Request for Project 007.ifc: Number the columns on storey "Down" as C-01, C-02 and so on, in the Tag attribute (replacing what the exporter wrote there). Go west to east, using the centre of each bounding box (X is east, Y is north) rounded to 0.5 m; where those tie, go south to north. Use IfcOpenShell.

First a look at what the model holds.

```python
import ifcopenshell
import ifcopenshell.util.element
import ifcopenshell.util.placement

model = ifcopenshell.open("Project 007.ifc")
print(model.schema)
storey = next(s for s in model.by_type("IfcBuildingStorey") if s.Name == "Down")
columns = [e for e in ifcopenshell.util.element.get_decomposition(storey) if e.is_a("IfcColumn")]
for e in sorted(columns, key=lambda e: e.id()):
    origin = ifcopenshell.util.placement.get_local_placement(e.ObjectPlacement)[:3, 3]
    print(e.id(), e.Tag, e.Name, origin.round(2) + 0.0, sep=" | ")
```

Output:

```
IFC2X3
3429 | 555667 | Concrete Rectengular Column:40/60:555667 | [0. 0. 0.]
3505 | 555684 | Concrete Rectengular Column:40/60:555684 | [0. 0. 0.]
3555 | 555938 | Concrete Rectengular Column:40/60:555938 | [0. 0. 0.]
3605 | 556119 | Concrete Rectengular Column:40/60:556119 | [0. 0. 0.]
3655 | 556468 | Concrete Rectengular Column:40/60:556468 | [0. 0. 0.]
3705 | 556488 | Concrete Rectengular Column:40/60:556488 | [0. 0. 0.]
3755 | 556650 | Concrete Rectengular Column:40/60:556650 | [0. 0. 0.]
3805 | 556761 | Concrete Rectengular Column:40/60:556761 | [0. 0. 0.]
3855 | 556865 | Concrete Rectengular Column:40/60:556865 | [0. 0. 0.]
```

```python
import ifcopenshell
import ifcopenshell.geom
import ifcopenshell.util.element
import ifcopenshell.util.shape

model = ifcopenshell.open("Project 007.ifc")
settings = ifcopenshell.geom.settings()
settings.set("use-world-coords", True)


def centre(element):
    shape = ifcopenshell.geom.create_shape(settings, element)
    return ifcopenshell.util.shape.get_bbox_centroid(shape.geometry)


storey = next(s for s in model.by_type("IfcBuildingStorey") if s.Name == "Down")
columns = [e for e in ifcopenshell.util.element.get_decomposition(storey) if e.is_a("IfcColumn")]

# Insertion points can sit at a corner or the storey origin, so sort by the geometry (in metres).
centres = {e: centre(e) for e in columns}
columns.sort(key=lambda e: (round(centres[e][0] / 0.5), centres[e][1]))

for i, e in enumerate(columns, start=1):
    number = f"C-{i:02d}"
    e.Tag = number
    print(e.id(), number)

model.write("Project 007_updated.ifc")
```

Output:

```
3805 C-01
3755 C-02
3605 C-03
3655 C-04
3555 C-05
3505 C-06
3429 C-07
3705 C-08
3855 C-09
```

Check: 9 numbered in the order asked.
